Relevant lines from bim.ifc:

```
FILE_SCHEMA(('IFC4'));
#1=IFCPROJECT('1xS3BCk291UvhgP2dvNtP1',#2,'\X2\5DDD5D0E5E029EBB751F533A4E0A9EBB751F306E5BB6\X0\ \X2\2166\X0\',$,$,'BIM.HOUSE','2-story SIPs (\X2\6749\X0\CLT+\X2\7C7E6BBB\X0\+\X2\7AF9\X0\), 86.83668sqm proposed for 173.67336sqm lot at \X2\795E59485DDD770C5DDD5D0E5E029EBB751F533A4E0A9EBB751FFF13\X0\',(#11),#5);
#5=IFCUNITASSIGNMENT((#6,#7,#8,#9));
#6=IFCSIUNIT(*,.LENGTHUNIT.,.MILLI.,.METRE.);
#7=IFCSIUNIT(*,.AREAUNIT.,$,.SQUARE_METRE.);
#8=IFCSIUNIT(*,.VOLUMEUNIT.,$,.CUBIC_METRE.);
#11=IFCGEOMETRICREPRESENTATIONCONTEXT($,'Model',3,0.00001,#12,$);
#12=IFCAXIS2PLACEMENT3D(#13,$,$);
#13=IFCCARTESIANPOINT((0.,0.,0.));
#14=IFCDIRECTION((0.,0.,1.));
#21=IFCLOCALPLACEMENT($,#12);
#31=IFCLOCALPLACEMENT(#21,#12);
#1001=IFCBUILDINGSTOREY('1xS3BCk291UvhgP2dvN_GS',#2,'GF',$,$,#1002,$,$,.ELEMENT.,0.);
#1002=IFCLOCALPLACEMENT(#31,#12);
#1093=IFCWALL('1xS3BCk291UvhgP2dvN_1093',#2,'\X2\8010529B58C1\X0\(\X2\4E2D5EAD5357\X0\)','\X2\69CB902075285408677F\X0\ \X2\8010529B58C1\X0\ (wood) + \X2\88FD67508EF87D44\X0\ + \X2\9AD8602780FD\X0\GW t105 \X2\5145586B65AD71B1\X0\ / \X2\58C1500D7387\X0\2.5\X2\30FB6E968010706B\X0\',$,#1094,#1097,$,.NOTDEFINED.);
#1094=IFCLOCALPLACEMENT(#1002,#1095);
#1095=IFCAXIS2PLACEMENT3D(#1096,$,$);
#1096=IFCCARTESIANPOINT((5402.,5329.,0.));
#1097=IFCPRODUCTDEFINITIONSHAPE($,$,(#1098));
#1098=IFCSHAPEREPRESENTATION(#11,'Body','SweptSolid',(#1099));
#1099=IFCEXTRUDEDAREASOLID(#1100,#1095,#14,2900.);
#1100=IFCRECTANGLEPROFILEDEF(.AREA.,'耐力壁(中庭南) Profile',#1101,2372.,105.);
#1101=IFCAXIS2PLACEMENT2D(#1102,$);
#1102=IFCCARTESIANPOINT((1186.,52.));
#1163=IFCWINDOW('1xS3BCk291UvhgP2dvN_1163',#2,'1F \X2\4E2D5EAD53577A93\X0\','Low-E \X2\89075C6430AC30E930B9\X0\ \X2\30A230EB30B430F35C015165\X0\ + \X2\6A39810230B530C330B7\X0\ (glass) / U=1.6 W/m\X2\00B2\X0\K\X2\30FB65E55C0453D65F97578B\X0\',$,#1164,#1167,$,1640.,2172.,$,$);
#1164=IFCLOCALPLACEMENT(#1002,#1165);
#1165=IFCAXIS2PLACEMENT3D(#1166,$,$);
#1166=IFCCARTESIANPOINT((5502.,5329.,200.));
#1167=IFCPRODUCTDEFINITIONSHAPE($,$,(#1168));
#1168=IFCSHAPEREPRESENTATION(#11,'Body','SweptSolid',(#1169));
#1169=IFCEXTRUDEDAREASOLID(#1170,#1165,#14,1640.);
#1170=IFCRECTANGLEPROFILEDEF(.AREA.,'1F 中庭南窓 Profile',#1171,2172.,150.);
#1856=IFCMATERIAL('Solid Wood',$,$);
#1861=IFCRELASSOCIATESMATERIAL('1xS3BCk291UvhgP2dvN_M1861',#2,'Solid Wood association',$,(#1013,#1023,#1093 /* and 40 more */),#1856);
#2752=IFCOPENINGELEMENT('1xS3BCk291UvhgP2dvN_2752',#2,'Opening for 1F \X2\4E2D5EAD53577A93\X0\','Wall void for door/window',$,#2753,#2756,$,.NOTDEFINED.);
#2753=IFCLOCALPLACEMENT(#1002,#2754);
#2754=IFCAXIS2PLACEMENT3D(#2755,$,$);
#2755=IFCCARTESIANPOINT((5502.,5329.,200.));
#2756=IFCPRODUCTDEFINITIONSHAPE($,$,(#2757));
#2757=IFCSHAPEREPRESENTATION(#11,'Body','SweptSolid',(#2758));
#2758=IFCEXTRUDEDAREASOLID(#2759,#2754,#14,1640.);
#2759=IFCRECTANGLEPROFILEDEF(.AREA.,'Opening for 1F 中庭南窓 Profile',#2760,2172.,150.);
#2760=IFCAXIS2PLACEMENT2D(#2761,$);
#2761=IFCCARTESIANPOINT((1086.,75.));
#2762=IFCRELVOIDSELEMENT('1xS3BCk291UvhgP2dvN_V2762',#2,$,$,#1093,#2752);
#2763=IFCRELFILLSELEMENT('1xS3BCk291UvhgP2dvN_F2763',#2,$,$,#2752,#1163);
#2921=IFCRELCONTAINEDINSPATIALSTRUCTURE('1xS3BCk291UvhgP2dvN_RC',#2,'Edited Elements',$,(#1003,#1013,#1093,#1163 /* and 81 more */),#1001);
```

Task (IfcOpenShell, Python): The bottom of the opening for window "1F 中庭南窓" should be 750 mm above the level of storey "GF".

```python
import numpy as np
import ifcopenshell
import ifcopenshell.api.geometry
import ifcopenshell.geom
import ifcopenshell.util.element
import ifcopenshell.util.placement
import ifcopenshell.util.shape
import ifcopenshell.util.unit

model = ifcopenshell.open("bim.ifc")
unit_scale = ifcopenshell.util.unit.calculate_unit_scale(model)

window = model.by_guid("1xS3BCk291UvhgP2dvN_1163")
opening = window.FillsVoids[0].RelatingOpeningElement
storey = ifcopenshell.util.element.get_container(window, ifc_class="IfcBuildingStorey")
level = ifcopenshell.util.placement.get_local_placement(storey.ObjectPlacement)[2, 3]

# The opening's origin need not be at the sill, so measure its lowest point.
shape = ifcopenshell.geom.create_shape(ifcopenshell.geom.settings(), opening)
bottom = ifcopenshell.util.shape.get_shape_bottom_elevation(shape, shape.geometry) / unit_scale
dz = level + 750.0 - bottom

shift = np.array([0.0, 0.0, dz])
# The window is not placed relative to its opening, so move both.
for product in (opening, window):
    matrix = ifcopenshell.util.placement.get_local_placement(product.ObjectPlacement)
    matrix[:3, 3] += shift
    ifcopenshell.api.geometry.edit_object_placement(model, product=product, matrix=matrix, is_si=False)

print(f"moved by {dz * unit_scale:+.3f} m")

model.write("bim_edited.ifc")
```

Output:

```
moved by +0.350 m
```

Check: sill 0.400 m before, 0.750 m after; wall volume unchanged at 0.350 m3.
